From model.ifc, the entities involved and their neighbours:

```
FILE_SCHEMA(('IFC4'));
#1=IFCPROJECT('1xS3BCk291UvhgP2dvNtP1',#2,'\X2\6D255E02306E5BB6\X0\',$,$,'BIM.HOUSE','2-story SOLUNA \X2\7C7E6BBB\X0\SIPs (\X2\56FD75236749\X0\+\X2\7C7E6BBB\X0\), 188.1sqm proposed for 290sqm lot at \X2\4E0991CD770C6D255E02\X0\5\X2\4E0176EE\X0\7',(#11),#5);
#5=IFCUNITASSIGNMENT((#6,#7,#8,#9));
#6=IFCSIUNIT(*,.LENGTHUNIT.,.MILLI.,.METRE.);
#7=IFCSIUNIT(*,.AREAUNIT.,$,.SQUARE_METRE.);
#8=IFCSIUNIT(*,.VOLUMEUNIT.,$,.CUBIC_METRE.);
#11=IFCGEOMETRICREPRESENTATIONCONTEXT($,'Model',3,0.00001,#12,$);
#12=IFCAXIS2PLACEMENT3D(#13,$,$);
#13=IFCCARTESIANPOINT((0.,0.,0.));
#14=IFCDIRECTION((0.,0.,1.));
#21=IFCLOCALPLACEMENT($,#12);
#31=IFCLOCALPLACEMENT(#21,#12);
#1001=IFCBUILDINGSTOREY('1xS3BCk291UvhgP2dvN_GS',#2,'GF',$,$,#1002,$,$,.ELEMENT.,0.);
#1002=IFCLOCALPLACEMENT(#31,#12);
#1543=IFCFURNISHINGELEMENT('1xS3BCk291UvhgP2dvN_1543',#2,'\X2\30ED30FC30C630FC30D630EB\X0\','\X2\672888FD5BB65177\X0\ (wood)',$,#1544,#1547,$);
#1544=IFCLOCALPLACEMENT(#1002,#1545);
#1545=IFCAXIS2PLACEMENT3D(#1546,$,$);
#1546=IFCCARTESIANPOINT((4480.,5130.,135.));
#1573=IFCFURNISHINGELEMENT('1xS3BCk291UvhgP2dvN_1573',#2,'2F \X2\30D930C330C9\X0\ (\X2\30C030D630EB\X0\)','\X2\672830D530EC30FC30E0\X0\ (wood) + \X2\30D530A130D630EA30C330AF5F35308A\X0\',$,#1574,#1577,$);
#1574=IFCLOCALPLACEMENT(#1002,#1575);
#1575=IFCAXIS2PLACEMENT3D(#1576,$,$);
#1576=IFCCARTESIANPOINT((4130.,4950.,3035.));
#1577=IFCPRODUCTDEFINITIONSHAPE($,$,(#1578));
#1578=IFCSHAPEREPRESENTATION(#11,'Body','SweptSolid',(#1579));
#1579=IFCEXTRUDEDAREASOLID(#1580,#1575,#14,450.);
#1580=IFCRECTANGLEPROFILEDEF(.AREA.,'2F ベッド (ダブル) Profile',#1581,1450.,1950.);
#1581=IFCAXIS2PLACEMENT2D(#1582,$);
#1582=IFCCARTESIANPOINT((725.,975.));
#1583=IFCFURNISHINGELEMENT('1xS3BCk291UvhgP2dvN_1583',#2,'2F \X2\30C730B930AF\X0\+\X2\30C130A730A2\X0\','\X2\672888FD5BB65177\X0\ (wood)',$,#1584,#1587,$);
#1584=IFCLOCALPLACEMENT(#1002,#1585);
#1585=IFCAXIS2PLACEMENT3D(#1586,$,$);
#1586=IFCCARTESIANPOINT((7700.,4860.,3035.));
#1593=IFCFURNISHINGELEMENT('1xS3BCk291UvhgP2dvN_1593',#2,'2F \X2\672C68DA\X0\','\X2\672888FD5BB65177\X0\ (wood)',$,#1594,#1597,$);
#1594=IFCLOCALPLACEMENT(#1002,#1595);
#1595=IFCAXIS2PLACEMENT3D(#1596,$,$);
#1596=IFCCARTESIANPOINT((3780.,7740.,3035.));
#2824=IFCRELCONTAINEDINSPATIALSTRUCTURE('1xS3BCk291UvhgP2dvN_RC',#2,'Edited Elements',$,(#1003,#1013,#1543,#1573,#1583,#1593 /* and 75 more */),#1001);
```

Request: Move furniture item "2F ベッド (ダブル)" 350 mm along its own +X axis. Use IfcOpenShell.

```python
import ifcopenshell
import ifcopenshell.api.geometry
import ifcopenshell.util.placement
import ifcopenshell.util.unit

model = ifcopenshell.open("model.ifc")
unit_scale = ifcopenshell.util.unit.calculate_unit_scale(model)

item = model.by_id(1573)
matrix = ifcopenshell.util.placement.get_local_placement(item.ObjectPlacement)
matrix[:3, 3] += matrix[:3, 0] * 0.35 / unit_scale
ifcopenshell.api.geometry.edit_object_placement(model, product=item, matrix=matrix, is_si=False)

print(ifcopenshell.util.placement.get_local_placement(item.ObjectPlacement).round(3) + 0.0)

model.write("model_updated.ifc")
```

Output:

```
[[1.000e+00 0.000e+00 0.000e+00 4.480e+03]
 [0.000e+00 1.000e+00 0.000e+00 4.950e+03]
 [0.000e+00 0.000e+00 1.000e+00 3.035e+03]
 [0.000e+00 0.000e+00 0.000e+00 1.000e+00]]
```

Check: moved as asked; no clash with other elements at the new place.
